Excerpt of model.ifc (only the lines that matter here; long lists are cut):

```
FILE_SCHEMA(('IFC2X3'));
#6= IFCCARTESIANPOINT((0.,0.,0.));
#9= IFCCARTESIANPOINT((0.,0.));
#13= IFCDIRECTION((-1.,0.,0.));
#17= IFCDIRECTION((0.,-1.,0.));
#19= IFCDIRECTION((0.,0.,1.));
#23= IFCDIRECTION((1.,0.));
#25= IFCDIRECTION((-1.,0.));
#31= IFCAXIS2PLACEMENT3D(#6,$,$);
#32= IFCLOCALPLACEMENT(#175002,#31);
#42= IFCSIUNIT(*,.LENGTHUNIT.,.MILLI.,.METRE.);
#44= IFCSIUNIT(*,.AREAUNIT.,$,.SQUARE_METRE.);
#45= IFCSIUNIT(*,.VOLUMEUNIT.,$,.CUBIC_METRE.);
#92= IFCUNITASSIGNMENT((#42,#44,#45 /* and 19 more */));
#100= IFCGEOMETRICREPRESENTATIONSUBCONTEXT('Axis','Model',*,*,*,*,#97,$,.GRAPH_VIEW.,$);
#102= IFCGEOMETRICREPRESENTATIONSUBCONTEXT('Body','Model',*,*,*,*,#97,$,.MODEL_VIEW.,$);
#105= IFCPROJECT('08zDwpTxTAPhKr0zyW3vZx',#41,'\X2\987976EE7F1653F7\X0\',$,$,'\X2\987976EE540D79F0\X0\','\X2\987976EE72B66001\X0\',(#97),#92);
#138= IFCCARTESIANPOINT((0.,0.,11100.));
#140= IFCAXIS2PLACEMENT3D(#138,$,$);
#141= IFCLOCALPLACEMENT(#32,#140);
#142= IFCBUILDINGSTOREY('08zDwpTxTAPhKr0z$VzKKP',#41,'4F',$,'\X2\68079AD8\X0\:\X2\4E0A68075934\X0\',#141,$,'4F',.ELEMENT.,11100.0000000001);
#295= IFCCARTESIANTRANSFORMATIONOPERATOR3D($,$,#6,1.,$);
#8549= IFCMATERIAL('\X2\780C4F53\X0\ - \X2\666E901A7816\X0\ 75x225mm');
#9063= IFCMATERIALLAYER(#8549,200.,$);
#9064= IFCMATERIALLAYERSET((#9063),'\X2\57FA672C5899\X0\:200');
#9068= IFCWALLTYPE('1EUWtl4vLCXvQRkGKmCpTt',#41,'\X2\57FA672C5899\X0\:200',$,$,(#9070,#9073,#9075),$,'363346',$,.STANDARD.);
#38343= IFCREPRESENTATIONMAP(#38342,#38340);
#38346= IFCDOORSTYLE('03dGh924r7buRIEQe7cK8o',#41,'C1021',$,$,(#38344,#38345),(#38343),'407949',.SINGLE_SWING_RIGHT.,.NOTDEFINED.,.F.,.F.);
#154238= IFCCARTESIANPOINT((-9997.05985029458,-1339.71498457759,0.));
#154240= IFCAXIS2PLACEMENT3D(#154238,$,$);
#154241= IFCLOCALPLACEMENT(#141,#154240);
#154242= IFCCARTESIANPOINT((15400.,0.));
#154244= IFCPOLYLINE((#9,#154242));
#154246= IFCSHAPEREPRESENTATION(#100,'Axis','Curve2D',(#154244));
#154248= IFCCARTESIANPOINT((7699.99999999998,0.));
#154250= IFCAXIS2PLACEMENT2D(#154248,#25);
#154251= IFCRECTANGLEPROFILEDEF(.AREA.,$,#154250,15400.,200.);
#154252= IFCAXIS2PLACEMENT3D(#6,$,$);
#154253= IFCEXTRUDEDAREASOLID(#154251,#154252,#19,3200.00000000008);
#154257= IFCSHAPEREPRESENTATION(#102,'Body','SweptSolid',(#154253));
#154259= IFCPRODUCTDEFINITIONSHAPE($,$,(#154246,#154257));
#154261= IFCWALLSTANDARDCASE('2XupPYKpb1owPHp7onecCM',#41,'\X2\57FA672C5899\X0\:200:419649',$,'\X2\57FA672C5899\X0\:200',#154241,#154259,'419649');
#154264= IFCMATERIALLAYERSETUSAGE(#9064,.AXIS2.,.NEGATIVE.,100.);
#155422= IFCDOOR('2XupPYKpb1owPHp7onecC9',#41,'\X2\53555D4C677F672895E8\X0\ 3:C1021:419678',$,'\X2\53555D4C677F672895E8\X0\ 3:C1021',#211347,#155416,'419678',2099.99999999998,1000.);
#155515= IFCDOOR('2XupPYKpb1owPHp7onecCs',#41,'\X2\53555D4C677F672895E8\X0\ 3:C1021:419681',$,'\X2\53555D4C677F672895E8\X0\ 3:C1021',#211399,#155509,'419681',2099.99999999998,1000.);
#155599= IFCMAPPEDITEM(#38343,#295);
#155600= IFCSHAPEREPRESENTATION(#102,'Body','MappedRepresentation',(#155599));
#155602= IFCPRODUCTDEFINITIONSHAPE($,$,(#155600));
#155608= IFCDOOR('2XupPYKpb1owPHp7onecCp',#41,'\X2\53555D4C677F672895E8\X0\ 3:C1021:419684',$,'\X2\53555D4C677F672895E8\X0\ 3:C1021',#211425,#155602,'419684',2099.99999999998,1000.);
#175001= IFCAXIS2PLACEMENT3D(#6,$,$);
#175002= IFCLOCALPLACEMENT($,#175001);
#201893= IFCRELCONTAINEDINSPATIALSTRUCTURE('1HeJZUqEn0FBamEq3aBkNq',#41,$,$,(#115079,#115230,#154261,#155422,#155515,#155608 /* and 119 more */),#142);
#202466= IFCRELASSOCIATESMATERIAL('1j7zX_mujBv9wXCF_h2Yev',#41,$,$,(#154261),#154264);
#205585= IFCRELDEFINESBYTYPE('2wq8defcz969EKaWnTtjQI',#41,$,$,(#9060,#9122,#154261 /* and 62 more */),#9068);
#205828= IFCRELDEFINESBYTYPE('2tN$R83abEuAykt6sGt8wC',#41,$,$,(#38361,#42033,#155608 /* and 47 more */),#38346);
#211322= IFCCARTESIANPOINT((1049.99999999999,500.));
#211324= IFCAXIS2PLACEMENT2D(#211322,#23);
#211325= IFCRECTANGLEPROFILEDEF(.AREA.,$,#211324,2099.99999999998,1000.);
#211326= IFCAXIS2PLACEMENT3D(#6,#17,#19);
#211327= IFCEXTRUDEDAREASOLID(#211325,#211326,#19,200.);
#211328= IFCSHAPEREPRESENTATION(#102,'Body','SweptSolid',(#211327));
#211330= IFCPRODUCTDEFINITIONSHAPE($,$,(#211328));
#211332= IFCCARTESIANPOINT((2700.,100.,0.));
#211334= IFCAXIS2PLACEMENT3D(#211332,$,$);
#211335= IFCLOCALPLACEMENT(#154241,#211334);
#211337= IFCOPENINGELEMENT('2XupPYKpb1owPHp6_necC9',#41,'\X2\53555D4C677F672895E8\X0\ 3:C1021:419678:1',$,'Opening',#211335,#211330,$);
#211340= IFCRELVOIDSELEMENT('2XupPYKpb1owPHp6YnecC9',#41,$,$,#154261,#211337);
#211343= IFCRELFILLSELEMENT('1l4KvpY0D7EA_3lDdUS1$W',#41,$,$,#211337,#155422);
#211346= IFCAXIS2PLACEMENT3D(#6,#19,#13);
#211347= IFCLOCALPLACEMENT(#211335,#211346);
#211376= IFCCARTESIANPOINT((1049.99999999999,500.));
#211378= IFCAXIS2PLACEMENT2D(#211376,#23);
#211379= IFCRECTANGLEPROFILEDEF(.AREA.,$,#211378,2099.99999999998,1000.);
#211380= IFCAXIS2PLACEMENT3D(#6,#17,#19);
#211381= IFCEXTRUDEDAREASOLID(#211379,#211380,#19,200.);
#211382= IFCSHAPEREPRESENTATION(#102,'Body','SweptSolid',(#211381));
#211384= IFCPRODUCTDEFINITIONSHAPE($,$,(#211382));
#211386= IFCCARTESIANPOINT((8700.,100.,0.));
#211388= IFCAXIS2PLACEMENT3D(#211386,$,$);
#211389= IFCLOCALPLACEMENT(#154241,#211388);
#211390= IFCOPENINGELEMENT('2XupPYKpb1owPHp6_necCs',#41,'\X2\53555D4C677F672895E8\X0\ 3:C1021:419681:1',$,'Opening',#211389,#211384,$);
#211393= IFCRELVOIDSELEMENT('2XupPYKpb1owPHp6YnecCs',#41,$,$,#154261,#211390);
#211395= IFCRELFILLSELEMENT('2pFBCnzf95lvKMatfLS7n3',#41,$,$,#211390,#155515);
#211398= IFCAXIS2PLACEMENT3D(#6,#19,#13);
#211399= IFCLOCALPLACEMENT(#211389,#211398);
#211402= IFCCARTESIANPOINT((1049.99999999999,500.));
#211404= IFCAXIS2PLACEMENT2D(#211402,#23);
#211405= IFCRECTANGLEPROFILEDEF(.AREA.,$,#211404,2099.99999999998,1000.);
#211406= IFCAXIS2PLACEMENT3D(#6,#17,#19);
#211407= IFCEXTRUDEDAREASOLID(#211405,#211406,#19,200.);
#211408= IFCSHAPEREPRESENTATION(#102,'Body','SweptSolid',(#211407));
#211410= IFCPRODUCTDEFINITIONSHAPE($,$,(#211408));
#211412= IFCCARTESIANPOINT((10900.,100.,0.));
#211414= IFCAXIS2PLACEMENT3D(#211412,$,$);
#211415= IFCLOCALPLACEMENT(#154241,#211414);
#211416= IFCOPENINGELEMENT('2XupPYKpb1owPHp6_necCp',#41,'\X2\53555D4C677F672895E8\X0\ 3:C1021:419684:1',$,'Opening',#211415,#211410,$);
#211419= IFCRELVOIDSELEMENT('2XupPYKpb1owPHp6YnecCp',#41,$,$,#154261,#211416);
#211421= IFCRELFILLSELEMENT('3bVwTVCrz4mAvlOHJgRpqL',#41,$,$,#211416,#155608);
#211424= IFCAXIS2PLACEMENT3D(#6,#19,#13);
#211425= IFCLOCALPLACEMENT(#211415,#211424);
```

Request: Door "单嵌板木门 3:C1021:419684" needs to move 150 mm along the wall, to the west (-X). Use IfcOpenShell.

```python
import ifcopenshell
import ifcopenshell.api.geometry
import ifcopenshell.util.placement
import ifcopenshell.util.unit

model = ifcopenshell.open("model.ifc")
unit_scale = ifcopenshell.util.unit.calculate_unit_scale(model)

door = model.by_guid("2XupPYKpb1owPHp7onecCp")
opening = door.FillsVoids[0].RelatingOpeningElement
wall = opening.VoidsElements[0].RelatingBuildingElement

wall_matrix = ifcopenshell.util.placement.get_local_placement(wall.ObjectPlacement)
shift = wall_matrix[:3, 0] * -0.15 / unit_scale
before = ifcopenshell.util.placement.get_local_placement(door.ObjectPlacement)[:3, 3].copy()

# The door is placed relative to its opening, so it follows when the opening moves.
matrix = ifcopenshell.util.placement.get_local_placement(opening.ObjectPlacement)
matrix[:3, 3] += shift
ifcopenshell.api.geometry.edit_object_placement(
    model, product=opening, matrix=matrix, is_si=False, should_transform_children=True
)

after = ifcopenshell.util.placement.get_local_placement(door.ObjectPlacement)[:3, 3]
print("door moved by", (after - before).round(3) + 0.0)

model.write("model_updated.ifc")
```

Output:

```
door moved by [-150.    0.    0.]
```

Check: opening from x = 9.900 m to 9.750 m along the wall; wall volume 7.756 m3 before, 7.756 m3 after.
